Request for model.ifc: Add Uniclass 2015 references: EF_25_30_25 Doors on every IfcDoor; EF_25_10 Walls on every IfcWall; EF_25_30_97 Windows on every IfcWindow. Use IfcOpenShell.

First a look at what the model holds.

```python
import ifcopenshell

model = ifcopenshell.open("model.ifc")
print(model.schema)
print("classifications:", [c.Name for c in model.by_type("IfcClassification")])
for ifc_class in ("IfcDoor", "IfcRoof", "IfcStair", "IfcWall", "IfcWindow"):
    print(ifc_class, len(model.by_type(ifc_class)))
```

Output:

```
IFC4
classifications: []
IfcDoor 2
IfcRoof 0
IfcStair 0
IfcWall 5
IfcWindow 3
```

```python
import ifcopenshell
import ifcopenshell.api.classification

model = ifcopenshell.open("model.ifc")

system = ifcopenshell.api.classification.add_classification(model, classification="Uniclass 2015")

codes = {
    "IfcDoor": ("EF_25_30_25", "Doors"),
    "IfcWall": ("EF_25_10", "Walls"),
    "IfcWindow": ("EF_25_30_97", "Windows"),
}
for ifc_class, (code, name) in codes.items():
    products = model.by_type(ifc_class)
    ifcopenshell.api.classification.add_reference(
        model, products=products, classification=system, identification=code, name=name
    )
    print(code, len(products))

model.write("model_rev.ifc")
```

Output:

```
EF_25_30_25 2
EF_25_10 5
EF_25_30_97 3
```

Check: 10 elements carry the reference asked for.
